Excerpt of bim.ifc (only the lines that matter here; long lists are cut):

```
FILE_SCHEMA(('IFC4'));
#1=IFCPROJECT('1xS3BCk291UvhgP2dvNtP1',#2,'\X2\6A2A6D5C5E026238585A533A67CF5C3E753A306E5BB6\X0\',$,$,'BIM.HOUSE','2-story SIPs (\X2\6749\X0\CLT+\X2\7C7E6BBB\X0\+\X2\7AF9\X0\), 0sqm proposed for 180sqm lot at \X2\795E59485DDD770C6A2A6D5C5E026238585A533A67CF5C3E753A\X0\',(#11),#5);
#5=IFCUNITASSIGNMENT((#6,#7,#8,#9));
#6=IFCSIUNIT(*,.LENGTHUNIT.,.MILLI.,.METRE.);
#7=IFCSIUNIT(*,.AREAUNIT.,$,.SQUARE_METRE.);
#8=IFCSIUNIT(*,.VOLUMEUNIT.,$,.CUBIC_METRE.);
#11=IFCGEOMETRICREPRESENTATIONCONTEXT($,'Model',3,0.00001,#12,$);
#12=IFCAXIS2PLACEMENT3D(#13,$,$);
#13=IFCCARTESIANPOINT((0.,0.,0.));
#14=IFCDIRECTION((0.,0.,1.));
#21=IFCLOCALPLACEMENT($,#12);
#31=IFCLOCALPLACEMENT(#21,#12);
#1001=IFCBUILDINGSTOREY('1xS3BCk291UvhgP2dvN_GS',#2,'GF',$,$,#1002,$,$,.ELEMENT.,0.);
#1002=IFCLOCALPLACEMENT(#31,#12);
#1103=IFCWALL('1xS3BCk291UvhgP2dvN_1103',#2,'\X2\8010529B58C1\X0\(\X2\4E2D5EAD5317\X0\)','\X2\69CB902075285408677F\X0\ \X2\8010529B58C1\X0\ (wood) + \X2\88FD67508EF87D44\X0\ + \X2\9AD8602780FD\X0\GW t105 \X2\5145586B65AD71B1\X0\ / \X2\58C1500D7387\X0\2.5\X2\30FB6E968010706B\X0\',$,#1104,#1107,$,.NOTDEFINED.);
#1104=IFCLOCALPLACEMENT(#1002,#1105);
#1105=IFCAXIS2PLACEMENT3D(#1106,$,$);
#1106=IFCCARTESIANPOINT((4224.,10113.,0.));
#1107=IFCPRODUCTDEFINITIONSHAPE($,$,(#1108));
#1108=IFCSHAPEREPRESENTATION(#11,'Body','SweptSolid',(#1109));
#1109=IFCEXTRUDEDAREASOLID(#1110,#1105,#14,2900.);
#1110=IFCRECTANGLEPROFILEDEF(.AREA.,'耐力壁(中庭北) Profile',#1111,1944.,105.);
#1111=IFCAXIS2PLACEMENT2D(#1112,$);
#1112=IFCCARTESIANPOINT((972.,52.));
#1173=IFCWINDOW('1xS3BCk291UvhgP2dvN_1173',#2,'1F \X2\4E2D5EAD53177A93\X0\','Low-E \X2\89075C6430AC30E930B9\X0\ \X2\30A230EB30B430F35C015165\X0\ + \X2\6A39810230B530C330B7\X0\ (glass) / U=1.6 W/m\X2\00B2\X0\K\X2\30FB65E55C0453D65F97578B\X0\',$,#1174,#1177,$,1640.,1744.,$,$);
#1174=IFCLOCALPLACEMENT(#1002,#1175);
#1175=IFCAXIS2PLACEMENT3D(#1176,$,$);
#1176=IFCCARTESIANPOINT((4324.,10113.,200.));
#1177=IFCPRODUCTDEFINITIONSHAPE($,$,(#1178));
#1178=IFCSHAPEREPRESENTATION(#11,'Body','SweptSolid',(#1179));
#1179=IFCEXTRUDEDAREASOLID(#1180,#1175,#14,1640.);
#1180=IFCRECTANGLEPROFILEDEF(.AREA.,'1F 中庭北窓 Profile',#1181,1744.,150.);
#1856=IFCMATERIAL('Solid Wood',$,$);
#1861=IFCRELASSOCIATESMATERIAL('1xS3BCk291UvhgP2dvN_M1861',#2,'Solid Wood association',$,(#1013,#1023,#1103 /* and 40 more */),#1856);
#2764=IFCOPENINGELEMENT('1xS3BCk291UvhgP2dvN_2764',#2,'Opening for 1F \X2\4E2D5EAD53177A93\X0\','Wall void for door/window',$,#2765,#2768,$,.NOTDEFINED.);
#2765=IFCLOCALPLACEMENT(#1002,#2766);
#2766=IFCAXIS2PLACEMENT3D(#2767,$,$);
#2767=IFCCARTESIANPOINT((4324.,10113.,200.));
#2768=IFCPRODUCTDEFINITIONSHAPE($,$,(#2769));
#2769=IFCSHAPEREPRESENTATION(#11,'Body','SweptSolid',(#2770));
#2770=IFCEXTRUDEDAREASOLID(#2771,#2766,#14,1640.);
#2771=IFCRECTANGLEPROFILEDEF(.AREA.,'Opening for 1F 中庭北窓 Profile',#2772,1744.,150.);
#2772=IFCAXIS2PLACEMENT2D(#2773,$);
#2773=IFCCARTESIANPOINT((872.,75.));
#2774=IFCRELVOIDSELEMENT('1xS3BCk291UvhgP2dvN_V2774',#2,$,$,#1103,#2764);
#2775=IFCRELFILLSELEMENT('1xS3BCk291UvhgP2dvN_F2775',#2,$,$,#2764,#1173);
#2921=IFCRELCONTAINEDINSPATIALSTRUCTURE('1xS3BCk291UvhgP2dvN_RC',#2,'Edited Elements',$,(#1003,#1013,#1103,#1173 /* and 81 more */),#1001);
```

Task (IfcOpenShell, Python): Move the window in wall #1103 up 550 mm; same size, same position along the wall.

```python
import numpy as np
import ifcopenshell
import ifcopenshell.api.geometry
import ifcopenshell.util.placement
import ifcopenshell.util.unit

model = ifcopenshell.open("bim.ifc")
unit_scale = ifcopenshell.util.unit.calculate_unit_scale(model)

window = model.by_guid("1xS3BCk291UvhgP2dvN_1173")
opening = window.FillsVoids[0].RelatingOpeningElement
dz = 550.0

shift = np.array([0.0, 0.0, dz])
# The window is not placed relative to its opening, so move both.
for product in (opening, window):
    matrix = ifcopenshell.util.placement.get_local_placement(product.ObjectPlacement)
    matrix[:3, 3] += shift
    ifcopenshell.api.geometry.edit_object_placement(model, product=product, matrix=matrix, is_si=False)

print(f"moved by {dz * unit_scale:+.3f} m")

model.write("bim_v2.ifc")
```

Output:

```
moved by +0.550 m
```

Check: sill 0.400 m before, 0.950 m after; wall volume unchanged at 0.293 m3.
